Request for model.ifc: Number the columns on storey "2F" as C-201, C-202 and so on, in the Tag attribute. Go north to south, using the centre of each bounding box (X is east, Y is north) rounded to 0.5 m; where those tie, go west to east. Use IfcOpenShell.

First a look at what the model holds.

```python
import ifcopenshell
import ifcopenshell.util.element
import ifcopenshell.util.placement

model = ifcopenshell.open("model.ifc")
print(model.schema)
storey = next(s for s in model.by_type("IfcBuildingStorey") if s.Name == "2F")
columns = [e for e in ifcopenshell.util.element.get_decomposition(storey) if e.is_a("IfcColumn")]
for e in sorted(columns, key=lambda e: e.id()):
    origin = ifcopenshell.util.placement.get_local_placement(e.ObjectPlacement)[:3, 3]
    print(e.id(), e.Tag, e.Name, origin.round(2) + 0.0, sep=" | ")
```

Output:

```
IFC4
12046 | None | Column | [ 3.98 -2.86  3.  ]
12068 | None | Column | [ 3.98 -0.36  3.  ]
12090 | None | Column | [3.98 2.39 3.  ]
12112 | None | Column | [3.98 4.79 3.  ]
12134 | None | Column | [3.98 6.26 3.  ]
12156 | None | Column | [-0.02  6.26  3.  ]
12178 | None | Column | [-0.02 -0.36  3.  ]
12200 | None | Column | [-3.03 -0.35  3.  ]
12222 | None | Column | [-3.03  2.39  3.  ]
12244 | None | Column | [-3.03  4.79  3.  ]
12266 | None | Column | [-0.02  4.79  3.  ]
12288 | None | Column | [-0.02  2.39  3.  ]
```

```python
import ifcopenshell
import ifcopenshell.geom
import ifcopenshell.util.element
import ifcopenshell.util.shape

model = ifcopenshell.open("model.ifc")
settings = ifcopenshell.geom.settings()
settings.set("use-world-coords", True)


def centre(element):
    shape = ifcopenshell.geom.create_shape(settings, element)
    return ifcopenshell.util.shape.get_bbox_centroid(shape.geometry)


storey = next(s for s in model.by_type("IfcBuildingStorey") if s.Name == "2F")
columns = [e for e in ifcopenshell.util.element.get_decomposition(storey) if e.is_a("IfcColumn")]

# Insertion points can sit at a corner or the storey origin, so sort by the geometry (in metres).
centres = {e: centre(e) for e in columns}
columns.sort(key=lambda e: (-round(centres[e][1] / 0.5), centres[e][0]))

for i, e in enumerate(columns, start=1):
    number = f"C-2{i:02d}"
    e.Tag = number
    print(e.id(), number)

model.write("model_rev.ifc")
```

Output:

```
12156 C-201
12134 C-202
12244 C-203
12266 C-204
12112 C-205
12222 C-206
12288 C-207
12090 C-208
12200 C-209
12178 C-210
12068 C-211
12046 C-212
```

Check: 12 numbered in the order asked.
